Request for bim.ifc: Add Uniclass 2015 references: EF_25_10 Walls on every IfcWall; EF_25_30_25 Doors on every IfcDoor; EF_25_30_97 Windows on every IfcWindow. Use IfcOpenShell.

First a look at what the model holds.

```python
import ifcopenshell

model = ifcopenshell.open("bim.ifc")
print(model.schema)
print("classifications:", [c.Name for c in model.by_type("IfcClassification")])
for ifc_class in ("IfcDoor", "IfcRoof", "IfcStair", "IfcWall", "IfcWindow"):
    print(ifc_class, len(model.by_type(ifc_class)))
```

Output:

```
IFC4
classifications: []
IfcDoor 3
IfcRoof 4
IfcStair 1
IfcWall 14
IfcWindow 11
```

```python
import ifcopenshell
import ifcopenshell.api.classification

model = ifcopenshell.open("bim.ifc")

system = ifcopenshell.api.classification.add_classification(model, classification="Uniclass 2015")

codes = {
    "IfcWall": ("EF_25_10", "Walls"),
    "IfcDoor": ("EF_25_30_25", "Doors"),
    "IfcWindow": ("EF_25_30_97", "Windows"),
}
for ifc_class, (code, name) in codes.items():
    products = model.by_type(ifc_class)
    ifcopenshell.api.classification.add_reference(
        model, products=products, classification=system, identification=code, name=name
    )
    print(code, len(products))

model.write("bim-out.ifc")
```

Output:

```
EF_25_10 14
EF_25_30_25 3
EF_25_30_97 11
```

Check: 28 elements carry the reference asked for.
